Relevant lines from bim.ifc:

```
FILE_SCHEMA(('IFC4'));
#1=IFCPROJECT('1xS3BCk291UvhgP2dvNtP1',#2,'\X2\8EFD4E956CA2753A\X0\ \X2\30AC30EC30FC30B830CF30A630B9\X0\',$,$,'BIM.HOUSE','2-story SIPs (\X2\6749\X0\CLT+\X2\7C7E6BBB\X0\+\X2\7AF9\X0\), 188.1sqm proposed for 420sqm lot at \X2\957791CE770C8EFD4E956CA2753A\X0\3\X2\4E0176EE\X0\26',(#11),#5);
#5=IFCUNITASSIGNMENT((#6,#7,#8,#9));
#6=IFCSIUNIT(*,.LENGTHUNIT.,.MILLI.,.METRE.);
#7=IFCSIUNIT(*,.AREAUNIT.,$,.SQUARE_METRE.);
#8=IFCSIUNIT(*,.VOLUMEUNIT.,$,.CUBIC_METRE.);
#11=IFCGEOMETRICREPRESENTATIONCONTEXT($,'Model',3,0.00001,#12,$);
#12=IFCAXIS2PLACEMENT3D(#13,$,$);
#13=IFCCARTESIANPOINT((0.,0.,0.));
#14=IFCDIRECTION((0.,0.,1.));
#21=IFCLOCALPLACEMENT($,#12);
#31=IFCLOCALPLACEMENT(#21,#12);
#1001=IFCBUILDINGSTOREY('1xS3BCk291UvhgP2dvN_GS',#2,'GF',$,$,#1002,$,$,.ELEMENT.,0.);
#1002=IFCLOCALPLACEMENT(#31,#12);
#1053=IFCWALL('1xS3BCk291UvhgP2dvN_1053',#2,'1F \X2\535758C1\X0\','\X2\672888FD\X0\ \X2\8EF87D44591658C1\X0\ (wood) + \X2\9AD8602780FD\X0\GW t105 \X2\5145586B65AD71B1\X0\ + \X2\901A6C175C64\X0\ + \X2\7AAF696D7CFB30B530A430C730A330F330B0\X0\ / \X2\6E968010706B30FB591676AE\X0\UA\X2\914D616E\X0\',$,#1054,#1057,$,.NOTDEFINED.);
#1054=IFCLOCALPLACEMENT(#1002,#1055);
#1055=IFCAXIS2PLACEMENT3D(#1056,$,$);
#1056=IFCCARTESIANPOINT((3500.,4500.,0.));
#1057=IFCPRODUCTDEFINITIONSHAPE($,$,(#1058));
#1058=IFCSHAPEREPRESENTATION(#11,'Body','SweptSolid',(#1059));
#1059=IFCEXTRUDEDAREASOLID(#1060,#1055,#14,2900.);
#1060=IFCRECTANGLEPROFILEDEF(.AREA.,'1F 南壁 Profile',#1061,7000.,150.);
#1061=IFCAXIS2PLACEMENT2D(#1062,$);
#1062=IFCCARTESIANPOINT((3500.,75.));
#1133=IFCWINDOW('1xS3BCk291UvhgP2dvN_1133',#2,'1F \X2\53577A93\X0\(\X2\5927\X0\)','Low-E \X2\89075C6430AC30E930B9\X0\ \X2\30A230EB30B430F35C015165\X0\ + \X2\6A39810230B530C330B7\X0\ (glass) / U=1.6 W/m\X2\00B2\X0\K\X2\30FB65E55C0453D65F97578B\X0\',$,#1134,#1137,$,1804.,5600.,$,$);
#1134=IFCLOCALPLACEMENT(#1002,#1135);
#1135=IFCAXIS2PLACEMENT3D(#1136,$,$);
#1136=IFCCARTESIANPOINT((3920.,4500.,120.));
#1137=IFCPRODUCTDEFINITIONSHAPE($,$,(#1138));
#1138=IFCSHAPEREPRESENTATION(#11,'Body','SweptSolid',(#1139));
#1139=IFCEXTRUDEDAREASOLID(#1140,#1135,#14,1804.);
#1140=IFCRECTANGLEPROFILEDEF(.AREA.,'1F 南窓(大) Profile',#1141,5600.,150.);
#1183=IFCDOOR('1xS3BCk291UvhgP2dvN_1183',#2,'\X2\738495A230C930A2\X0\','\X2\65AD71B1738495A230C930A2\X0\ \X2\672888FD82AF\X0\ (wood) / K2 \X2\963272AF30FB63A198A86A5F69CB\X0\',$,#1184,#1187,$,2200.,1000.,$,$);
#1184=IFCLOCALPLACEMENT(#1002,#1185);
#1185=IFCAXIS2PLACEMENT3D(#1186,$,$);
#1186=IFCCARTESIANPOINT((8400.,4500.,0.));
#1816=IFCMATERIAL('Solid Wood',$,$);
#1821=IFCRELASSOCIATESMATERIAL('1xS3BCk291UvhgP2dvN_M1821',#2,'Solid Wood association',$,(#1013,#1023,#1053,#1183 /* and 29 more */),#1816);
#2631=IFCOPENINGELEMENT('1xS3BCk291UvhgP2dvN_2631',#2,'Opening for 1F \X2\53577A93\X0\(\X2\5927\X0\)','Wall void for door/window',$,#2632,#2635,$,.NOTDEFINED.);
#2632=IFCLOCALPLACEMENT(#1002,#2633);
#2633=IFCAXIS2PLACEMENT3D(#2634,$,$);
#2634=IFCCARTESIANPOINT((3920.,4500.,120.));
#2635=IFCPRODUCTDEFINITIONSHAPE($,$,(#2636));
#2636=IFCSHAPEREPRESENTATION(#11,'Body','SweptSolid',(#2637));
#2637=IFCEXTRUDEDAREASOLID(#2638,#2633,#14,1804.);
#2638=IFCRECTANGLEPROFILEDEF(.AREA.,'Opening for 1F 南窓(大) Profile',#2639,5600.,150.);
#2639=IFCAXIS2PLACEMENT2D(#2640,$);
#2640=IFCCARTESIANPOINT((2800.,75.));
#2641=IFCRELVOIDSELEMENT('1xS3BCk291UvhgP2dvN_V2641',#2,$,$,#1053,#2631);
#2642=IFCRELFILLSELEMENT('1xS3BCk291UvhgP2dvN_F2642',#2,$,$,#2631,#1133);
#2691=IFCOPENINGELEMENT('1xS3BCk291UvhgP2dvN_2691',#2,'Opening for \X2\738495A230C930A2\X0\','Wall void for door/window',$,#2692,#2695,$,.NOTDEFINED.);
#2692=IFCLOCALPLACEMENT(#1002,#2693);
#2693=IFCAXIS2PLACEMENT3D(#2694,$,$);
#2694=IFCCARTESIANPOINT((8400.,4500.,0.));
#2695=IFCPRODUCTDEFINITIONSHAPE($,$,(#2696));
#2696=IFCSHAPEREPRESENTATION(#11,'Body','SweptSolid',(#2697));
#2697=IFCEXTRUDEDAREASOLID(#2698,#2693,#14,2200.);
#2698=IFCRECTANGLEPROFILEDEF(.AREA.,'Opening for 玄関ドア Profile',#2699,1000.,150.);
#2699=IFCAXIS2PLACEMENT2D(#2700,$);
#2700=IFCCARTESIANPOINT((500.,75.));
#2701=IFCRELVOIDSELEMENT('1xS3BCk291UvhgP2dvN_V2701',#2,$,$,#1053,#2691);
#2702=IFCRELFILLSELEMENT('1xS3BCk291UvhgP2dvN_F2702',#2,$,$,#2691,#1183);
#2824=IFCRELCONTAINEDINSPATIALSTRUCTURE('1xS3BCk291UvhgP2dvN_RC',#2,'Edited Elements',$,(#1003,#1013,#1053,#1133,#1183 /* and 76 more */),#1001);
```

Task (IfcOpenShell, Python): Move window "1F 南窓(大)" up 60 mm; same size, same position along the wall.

```python
import numpy as np
import ifcopenshell
import ifcopenshell.api.geometry
import ifcopenshell.util.placement
import ifcopenshell.util.unit

model = ifcopenshell.open("bim.ifc")
unit_scale = ifcopenshell.util.unit.calculate_unit_scale(model)

window = model.by_guid("1xS3BCk291UvhgP2dvN_1133")
opening = window.FillsVoids[0].RelatingOpeningElement
dz = 60.0

shift = np.array([0.0, 0.0, dz])
# The window is not placed relative to its opening, so move both.
for product in (opening, window):
    matrix = ifcopenshell.util.placement.get_local_placement(product.ObjectPlacement)
    matrix[:3, 3] += shift
    ifcopenshell.api.geometry.edit_object_placement(model, product=product, matrix=matrix, is_si=False)

print(f"moved by {dz * unit_scale:+.3f} m")

model.write("bim-out.ifc")
```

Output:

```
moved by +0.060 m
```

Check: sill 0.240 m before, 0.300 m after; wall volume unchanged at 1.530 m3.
